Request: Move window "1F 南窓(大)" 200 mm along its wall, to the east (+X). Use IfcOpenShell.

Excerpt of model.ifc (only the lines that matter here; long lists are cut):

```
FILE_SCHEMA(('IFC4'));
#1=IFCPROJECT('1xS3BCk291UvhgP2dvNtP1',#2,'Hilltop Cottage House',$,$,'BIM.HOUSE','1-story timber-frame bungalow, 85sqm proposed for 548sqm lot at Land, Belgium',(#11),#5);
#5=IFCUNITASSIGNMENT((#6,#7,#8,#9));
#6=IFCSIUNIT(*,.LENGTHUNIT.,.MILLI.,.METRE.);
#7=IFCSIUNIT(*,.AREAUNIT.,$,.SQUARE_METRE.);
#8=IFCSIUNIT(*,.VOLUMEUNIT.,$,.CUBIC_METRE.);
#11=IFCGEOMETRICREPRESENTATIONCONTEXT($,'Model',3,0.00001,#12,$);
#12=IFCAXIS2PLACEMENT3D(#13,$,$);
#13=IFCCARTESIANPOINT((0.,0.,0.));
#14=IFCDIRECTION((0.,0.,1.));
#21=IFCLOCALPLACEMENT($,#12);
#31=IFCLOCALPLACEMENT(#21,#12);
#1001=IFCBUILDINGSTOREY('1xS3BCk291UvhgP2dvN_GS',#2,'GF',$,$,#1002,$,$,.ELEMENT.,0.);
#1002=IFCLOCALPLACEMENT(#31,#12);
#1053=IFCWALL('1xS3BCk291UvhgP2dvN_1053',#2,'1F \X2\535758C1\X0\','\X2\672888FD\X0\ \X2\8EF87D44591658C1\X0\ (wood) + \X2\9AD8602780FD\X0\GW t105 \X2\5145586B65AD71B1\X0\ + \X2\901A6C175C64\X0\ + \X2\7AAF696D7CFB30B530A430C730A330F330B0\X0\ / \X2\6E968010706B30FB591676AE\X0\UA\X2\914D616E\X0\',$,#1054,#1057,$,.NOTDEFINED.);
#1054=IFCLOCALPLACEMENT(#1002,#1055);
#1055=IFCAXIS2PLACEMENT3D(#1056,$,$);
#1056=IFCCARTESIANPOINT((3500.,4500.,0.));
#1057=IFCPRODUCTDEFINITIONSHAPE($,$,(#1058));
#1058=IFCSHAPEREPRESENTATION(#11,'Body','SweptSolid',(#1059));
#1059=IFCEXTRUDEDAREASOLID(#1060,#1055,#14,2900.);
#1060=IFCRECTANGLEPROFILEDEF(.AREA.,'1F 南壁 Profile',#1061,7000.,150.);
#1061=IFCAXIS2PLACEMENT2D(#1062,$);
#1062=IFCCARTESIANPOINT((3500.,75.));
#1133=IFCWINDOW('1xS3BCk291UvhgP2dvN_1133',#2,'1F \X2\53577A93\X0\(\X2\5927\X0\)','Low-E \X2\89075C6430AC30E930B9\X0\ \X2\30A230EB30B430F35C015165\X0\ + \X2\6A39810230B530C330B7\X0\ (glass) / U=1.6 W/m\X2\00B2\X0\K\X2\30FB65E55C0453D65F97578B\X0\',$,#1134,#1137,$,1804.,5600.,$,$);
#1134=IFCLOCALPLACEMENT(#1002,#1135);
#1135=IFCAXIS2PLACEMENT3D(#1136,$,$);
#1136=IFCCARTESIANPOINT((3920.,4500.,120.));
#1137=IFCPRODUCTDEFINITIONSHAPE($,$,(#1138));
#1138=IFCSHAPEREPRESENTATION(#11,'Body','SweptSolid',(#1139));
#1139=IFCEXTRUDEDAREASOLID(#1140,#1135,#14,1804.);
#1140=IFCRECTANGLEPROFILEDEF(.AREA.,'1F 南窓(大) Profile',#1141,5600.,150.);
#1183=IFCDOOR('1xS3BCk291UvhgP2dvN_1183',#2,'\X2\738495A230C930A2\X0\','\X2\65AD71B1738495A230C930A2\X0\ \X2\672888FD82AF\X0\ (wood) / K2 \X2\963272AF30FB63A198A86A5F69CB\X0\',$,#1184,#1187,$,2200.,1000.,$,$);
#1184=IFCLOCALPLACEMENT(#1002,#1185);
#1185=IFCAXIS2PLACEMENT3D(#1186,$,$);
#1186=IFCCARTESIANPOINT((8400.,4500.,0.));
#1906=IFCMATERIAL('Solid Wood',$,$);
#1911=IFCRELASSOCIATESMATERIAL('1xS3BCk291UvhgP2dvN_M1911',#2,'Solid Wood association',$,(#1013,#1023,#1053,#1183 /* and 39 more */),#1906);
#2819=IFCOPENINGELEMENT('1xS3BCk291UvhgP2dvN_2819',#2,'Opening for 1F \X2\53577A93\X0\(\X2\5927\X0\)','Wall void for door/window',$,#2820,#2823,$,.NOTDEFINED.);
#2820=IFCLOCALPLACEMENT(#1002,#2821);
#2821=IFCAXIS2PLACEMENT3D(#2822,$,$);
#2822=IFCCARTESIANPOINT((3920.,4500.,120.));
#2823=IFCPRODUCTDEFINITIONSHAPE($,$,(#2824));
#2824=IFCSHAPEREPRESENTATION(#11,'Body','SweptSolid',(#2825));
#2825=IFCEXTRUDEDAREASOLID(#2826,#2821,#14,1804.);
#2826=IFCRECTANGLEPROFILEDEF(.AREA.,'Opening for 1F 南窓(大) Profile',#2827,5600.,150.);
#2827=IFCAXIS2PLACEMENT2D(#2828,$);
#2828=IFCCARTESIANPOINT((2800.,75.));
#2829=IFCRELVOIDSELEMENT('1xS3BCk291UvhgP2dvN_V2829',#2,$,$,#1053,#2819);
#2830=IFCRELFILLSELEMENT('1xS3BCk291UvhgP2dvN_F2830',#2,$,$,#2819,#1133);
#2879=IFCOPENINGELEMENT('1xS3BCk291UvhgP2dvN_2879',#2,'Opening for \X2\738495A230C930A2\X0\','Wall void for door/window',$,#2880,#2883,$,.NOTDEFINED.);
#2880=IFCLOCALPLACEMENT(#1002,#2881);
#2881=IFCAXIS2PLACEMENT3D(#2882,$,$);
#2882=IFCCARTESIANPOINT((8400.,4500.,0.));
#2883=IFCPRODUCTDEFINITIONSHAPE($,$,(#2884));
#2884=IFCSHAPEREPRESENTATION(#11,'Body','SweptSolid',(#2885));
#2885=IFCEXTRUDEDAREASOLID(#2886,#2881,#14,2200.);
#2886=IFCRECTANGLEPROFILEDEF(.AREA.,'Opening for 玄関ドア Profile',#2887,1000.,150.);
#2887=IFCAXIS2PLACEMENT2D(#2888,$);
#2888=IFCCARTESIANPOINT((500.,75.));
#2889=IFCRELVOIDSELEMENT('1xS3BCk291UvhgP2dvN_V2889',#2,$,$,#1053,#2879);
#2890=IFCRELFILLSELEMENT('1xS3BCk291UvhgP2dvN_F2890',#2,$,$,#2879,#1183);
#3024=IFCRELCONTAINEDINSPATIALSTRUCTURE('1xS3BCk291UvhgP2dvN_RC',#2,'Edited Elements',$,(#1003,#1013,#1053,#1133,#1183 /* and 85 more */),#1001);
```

```python
import ifcopenshell
import ifcopenshell.api.geometry
import ifcopenshell.util.placement

model = ifcopenshell.open("model.ifc")

window = model.by_id(1133)
opening = window.FillsVoids[0].RelatingOpeningElement
wall = opening.VoidsElements[0].RelatingBuildingElement

wall_matrix = ifcopenshell.util.placement.get_local_placement(wall.ObjectPlacement)
shift = wall_matrix[:3, 0] * 200.0
before = ifcopenshell.util.placement.get_local_placement(window.ObjectPlacement)[:3, 3].copy()

# The window is not placed relative to its opening, so move both.
for product in (opening, window):
    matrix = ifcopenshell.util.placement.get_local_placement(product.ObjectPlacement)
    matrix[:3, 3] += shift
    ifcopenshell.api.geometry.edit_object_placement(model, product=product, matrix=matrix, is_si=False)

after = ifcopenshell.util.placement.get_local_placement(window.ObjectPlacement)[:3, 3]
print("window moved by", (after - before).round(3) + 0.0)

model.write("model-out.ifc")
```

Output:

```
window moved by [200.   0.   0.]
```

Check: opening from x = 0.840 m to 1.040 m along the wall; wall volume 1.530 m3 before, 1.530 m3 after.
